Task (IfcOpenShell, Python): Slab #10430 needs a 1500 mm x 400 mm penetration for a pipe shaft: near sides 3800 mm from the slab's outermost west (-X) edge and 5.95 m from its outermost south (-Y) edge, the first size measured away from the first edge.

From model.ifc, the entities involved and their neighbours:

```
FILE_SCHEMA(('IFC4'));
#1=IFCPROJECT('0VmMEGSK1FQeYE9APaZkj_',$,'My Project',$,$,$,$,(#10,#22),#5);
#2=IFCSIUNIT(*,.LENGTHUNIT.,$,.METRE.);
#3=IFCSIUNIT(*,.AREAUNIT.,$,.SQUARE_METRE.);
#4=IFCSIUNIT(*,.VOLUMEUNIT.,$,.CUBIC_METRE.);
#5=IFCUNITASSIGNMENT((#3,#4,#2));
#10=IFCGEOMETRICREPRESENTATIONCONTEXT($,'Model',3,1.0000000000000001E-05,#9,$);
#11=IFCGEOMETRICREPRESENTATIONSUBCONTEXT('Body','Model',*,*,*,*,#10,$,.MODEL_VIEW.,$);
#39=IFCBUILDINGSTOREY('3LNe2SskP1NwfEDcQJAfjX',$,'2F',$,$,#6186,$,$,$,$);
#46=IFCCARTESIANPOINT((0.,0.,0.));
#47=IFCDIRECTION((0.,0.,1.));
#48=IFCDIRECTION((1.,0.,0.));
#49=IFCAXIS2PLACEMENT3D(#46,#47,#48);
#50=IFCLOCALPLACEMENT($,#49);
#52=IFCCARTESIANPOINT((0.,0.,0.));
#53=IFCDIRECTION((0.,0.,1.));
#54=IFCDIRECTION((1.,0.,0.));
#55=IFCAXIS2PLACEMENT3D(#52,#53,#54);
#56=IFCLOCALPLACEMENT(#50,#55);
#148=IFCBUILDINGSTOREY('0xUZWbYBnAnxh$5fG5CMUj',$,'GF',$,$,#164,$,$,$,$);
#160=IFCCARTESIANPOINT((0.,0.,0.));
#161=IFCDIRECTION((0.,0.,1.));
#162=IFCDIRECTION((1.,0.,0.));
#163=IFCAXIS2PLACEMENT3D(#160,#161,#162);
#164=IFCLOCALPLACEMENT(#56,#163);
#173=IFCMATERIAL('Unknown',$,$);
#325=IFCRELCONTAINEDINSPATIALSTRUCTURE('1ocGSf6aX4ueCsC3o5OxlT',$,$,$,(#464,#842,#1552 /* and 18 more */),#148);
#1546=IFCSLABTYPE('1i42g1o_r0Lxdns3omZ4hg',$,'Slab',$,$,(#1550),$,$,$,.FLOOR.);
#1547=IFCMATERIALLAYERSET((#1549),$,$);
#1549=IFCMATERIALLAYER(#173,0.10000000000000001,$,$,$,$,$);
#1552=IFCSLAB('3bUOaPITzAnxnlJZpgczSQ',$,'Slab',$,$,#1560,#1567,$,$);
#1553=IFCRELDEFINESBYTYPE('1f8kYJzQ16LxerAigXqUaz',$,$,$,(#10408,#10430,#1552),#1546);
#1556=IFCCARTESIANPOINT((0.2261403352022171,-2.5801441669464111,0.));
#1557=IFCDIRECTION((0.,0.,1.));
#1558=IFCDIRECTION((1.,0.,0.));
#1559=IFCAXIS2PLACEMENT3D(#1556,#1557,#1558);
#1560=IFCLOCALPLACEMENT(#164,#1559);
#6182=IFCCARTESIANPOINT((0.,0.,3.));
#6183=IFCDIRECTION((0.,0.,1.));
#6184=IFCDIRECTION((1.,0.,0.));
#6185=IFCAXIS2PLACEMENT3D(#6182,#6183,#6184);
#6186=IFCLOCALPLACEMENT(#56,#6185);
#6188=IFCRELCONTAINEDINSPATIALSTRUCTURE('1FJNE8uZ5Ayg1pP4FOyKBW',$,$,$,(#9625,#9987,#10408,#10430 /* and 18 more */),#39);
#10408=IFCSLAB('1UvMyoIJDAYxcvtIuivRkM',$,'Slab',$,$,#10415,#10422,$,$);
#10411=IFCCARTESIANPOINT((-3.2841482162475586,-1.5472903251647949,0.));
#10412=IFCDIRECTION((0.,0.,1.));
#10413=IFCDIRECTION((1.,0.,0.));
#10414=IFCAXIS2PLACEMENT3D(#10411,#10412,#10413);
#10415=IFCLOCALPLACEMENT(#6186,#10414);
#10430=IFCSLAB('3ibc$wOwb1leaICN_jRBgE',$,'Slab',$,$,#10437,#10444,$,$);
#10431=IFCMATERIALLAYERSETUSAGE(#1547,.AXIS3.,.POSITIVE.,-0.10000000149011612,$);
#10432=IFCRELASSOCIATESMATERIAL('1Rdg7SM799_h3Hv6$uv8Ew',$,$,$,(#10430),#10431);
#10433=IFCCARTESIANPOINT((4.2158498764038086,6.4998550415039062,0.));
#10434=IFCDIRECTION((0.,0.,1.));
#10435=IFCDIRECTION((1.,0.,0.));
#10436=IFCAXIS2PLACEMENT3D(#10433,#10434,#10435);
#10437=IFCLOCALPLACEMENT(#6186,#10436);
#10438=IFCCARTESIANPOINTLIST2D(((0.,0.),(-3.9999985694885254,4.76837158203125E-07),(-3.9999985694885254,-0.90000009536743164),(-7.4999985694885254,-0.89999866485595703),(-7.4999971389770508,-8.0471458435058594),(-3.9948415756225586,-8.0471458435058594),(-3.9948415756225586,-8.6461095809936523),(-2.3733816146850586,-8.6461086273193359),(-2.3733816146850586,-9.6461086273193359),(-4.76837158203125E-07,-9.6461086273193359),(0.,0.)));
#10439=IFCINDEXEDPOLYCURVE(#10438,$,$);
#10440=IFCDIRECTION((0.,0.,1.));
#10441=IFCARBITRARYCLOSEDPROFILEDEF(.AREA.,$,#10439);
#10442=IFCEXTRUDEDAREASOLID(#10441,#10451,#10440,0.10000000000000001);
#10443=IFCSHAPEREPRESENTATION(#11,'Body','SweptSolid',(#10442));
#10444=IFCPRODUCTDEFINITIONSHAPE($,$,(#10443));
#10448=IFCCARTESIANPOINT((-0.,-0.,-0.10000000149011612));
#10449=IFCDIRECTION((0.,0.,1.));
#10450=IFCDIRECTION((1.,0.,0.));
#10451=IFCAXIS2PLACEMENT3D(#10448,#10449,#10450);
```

```python
import numpy as np
import ifcopenshell
import ifcopenshell.api.feature
import ifcopenshell.api.geometry
import ifcopenshell.api.root
import ifcopenshell.geom
import ifcopenshell.util.placement
import ifcopenshell.util.representation
import ifcopenshell.util.shape
import ifcopenshell.util.unit

model = ifcopenshell.open("model.ifc")
unit_scale = ifcopenshell.util.unit.calculate_unit_scale(model)
settings = ifcopenshell.geom.settings()


def volume(element):
    """Net volume in cubic metres, openings subtracted."""
    shape = ifcopenshell.geom.create_shape(settings, element)
    return ifcopenshell.util.shape.get_volume(shape.geometry)


slab = model.by_id(10430)
before = volume(slab)

# Extent in the slab's own axes, in metres. The edges named are its -X and -Y sides.
slab_shape = ifcopenshell.geom.create_shape(settings, slab)
vertices = ifcopenshell.util.shape.get_vertices(slab_shape.geometry)
x_min, y_min, bottom = vertices.min(axis=0)
top = vertices[:, 2].max()

opening = ifcopenshell.api.root.create_entity(model, ifc_class="IfcOpeningElement", name="Pipe shaft opening", predefined_type="OPENING")
context = ifcopenshell.util.representation.get_context(model, "Model", "Body", "MODEL_VIEW")
width, depth = 1.5, 0.4
outline = [(0.0, 0.0), (width, 0.0), (width, depth), (0.0, depth), (0.0, 0.0)]
# Overshoot both faces by 50 mm so the cut is clean.
shape = ifcopenshell.api.geometry.add_slab_representation(
    model, context=context, depth=top - bottom + 0.1, polyline=outline
)
ifcopenshell.api.geometry.assign_representation(model, product=opening, representation=shape)

matrix = ifcopenshell.util.placement.get_local_placement(slab.ObjectPlacement)
matrix[:, 3] = matrix @ np.append(np.array([x_min + 3.8, y_min + 5.95, bottom - 0.05]) / unit_scale, 1.0)
ifcopenshell.api.geometry.edit_object_placement(model, product=opening, matrix=matrix, is_si=False)
ifcopenshell.api.feature.add_feature(model, feature=opening, element=slab)

after = volume(slab)

print(f"slab volume {before:.3f} -> {after:.3f} m3")

model.write("model_rev.ifc")
```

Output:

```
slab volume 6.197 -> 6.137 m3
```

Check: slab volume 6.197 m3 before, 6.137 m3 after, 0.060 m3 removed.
